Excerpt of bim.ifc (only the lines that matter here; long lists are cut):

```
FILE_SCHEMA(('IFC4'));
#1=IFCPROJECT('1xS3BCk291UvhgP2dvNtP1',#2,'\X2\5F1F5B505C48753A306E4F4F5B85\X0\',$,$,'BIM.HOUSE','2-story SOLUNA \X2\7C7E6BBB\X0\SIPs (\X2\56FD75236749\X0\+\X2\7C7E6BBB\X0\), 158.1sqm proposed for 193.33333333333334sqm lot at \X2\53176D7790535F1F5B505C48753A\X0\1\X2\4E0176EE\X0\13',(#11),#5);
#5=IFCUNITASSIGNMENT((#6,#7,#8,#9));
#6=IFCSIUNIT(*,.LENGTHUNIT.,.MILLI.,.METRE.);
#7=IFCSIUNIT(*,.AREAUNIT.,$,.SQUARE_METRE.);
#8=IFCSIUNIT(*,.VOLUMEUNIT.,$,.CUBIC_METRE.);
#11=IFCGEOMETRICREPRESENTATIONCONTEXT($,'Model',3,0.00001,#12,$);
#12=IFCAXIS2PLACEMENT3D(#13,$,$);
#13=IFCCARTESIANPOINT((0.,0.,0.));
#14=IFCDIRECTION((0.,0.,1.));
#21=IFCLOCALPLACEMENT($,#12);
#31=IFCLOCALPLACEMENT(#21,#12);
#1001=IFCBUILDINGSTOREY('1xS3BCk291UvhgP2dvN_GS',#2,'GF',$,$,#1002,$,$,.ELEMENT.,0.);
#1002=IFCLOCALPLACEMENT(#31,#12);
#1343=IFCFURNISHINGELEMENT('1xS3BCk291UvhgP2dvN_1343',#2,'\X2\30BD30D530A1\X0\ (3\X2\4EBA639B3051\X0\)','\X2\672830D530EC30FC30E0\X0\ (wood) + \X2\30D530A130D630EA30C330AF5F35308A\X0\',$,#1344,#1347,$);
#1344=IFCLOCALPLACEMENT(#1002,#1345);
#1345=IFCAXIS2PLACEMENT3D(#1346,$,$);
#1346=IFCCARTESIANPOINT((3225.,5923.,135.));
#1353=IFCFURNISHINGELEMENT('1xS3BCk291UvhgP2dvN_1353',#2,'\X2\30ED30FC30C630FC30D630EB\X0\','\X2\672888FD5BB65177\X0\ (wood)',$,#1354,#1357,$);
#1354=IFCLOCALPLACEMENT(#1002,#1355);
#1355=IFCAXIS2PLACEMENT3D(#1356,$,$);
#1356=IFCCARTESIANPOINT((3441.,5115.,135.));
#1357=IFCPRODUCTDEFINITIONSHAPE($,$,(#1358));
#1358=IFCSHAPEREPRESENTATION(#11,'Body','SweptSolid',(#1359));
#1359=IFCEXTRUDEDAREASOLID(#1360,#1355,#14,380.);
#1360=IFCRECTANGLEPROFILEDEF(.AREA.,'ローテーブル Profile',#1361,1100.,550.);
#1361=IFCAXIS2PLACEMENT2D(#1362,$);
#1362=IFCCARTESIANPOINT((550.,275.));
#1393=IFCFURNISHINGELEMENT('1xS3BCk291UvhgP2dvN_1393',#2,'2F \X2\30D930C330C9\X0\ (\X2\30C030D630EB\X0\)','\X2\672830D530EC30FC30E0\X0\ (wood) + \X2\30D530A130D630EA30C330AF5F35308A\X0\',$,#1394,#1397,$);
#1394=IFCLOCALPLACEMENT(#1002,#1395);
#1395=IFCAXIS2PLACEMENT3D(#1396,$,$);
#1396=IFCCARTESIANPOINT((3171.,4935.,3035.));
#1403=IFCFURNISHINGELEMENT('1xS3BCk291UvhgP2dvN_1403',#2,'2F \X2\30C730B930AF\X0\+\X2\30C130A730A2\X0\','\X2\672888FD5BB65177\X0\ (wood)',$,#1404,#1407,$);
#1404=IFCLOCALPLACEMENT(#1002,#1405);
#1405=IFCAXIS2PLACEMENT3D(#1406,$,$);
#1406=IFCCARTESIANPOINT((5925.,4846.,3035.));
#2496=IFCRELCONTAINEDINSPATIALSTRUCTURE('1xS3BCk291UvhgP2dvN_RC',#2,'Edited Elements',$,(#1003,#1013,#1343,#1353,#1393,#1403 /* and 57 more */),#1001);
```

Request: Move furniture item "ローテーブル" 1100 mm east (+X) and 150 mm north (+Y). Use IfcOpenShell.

```python
import ifcopenshell
import ifcopenshell.api.geometry
import ifcopenshell.util.placement

model = ifcopenshell.open("bim.ifc")

item = model.by_guid("1xS3BCk291UvhgP2dvN_1353")
matrix = ifcopenshell.util.placement.get_local_placement(item.ObjectPlacement)
matrix[0, 3] += 1100.0
matrix[1, 3] += 150.0
ifcopenshell.api.geometry.edit_object_placement(model, product=item, matrix=matrix, is_si=False)

print(ifcopenshell.util.placement.get_local_placement(item.ObjectPlacement).round(3) + 0.0)

model.write("bim_rev.ifc")
```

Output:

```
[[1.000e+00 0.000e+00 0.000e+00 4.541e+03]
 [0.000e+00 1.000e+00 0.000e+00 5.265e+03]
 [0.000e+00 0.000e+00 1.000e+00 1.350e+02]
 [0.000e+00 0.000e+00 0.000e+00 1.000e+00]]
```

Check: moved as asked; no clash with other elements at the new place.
